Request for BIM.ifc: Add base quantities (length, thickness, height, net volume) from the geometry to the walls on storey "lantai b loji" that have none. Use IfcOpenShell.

First a look at what the model holds.

```python
import ifcopenshell
import ifcopenshell.util.element
import ifcopenshell.util.unit

model = ifcopenshell.open("BIM.ifc")
print(model.schema)
for unit_type in ("LENGTHUNIT", "AREAUNIT", "VOLUMEUNIT"):
    print(unit_type, ifcopenshell.util.unit.calculate_unit_scale(model, unit_type))
storey = next(s for s in model.by_type("IfcBuildingStorey") if s.Name == "lantai b loji")
walls = [e for e in ifcopenshell.util.element.get_decomposition(storey) if e.is_a("IfcWall")]
for e in sorted(walls, key=lambda e: e.id()):
    print(e.id(), e.is_a(), e.Name, list(ifcopenshell.util.element.get_psets(e, qtos_only=True)), sep=" | ")
```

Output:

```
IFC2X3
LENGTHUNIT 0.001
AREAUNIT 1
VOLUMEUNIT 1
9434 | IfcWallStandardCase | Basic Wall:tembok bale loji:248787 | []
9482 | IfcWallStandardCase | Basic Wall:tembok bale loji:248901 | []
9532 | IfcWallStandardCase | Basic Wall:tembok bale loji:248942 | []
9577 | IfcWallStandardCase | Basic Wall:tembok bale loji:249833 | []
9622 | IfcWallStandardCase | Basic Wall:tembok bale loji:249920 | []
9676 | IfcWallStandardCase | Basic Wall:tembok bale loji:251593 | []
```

```python
import ifcopenshell
import ifcopenshell.api.pset
import ifcopenshell.geom
import ifcopenshell.util.element
import ifcopenshell.util.shape
import ifcopenshell.util.unit

model = ifcopenshell.open("BIM.ifc")
unit_scale = ifcopenshell.util.unit.calculate_unit_scale(model)
volume_scale = ifcopenshell.util.unit.calculate_unit_scale(model, "VOLUMEUNIT")
settings = ifcopenshell.geom.settings()

storey = next(s for s in model.by_type("IfcBuildingStorey") if s.Name == "lantai b loji")
walls = [e for e in ifcopenshell.util.element.get_decomposition(storey) if e.is_a("IfcWall")]

for e in sorted(walls, key=lambda e: e.id()):
    if ifcopenshell.util.element.get_psets(e, qtos_only=True, should_inherit=False):
        continue
    # Geometry comes back in metres, in the element's own axes.
    shape = ifcopenshell.geom.create_shape(settings, e)
    values = {
        "Length": ifcopenshell.util.shape.get_x(shape.geometry) / unit_scale,
        "Width": ifcopenshell.util.shape.get_y(shape.geometry) / unit_scale,
        "Height": ifcopenshell.util.shape.get_z(shape.geometry) / unit_scale,
        "NetVolume": ifcopenshell.util.shape.get_volume(shape.geometry) / volume_scale,
    }
    qto = ifcopenshell.api.pset.add_qto(model, product=e, name="BaseQuantities")
    ifcopenshell.api.pset.edit_qto(model, qto=qto, properties=values)
    print(e.id(), {k: round(v, 3) for k, v in values.items()})

model.write("BIM_v2.ifc")
```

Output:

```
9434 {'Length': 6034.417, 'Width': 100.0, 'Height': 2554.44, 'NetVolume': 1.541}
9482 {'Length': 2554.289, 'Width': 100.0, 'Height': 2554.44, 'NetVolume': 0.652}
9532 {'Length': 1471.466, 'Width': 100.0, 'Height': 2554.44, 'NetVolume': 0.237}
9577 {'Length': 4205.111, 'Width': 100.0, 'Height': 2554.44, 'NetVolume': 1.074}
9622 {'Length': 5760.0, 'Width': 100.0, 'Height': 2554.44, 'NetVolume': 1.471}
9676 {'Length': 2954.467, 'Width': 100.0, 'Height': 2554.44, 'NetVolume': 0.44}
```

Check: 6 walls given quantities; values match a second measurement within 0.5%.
